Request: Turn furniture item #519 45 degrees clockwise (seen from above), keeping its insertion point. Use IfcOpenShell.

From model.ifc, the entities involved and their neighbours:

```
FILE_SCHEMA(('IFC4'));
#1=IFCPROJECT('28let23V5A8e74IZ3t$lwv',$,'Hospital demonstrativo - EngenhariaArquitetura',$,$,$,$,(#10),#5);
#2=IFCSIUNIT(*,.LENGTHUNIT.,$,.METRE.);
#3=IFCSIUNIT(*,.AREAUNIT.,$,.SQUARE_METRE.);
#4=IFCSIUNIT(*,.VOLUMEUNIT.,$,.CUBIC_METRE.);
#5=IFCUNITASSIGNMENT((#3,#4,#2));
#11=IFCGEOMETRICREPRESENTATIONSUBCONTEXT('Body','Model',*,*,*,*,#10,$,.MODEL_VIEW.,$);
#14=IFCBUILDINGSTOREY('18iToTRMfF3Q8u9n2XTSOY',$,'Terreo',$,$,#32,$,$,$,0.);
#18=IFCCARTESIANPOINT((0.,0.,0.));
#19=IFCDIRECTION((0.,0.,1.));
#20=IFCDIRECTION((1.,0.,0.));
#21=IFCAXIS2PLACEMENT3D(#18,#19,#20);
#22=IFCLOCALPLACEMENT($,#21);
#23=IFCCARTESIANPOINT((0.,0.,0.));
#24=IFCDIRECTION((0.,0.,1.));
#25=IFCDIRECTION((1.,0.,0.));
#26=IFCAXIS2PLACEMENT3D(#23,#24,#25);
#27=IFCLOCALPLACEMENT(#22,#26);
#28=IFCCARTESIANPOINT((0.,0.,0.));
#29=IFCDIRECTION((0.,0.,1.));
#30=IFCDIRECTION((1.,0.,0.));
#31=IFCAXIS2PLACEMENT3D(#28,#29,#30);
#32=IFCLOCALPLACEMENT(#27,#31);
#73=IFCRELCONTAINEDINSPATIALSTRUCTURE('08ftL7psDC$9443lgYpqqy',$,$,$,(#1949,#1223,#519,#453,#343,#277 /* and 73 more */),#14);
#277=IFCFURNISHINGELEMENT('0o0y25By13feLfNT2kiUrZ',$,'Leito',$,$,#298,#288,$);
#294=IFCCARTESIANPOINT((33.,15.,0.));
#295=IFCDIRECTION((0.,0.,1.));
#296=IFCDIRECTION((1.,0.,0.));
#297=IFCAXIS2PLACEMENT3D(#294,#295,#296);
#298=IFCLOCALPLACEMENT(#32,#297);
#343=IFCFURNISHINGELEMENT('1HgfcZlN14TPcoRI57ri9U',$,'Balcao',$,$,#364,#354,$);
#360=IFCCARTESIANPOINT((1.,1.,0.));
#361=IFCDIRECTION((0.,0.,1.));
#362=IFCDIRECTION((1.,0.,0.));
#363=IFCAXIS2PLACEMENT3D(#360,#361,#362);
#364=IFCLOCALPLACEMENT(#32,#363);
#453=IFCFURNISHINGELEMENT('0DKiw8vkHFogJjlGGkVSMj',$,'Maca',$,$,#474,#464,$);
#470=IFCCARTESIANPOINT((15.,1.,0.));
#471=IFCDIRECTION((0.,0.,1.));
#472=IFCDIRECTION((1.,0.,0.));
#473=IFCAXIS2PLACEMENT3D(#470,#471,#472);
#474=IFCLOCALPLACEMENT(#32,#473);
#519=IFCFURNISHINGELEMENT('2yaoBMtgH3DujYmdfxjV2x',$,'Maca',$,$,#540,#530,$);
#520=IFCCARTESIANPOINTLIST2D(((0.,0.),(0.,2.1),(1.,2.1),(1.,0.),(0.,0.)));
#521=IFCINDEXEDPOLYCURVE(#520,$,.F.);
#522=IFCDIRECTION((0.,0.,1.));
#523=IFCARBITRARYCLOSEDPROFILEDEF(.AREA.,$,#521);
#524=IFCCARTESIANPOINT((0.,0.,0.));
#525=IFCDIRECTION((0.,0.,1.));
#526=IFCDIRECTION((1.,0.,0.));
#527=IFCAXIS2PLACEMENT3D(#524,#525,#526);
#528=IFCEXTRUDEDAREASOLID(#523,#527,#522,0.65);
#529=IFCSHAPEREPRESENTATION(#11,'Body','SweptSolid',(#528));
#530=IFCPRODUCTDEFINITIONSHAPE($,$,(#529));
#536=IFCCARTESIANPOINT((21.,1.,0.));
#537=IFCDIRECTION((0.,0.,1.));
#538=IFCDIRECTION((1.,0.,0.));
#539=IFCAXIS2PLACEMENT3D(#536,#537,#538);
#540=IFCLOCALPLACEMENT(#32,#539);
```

```python
import ifcopenshell
import ifcopenshell.api.geometry
import ifcopenshell.util.placement

model = ifcopenshell.open("model.ifc")

item = model.by_id(519)
matrix = ifcopenshell.util.placement.get_local_placement(item.ObjectPlacement)
matrix = matrix @ ifcopenshell.util.placement.rotation(-45, "Z")
ifcopenshell.api.geometry.edit_object_placement(model, product=item, matrix=matrix, is_si=False)

print(ifcopenshell.util.placement.get_local_placement(item.ObjectPlacement).round(3) + 0.0)

model.write("model-out.ifc")
```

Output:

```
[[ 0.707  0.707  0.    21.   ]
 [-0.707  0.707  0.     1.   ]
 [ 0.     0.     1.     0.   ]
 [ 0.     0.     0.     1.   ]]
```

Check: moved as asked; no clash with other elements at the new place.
